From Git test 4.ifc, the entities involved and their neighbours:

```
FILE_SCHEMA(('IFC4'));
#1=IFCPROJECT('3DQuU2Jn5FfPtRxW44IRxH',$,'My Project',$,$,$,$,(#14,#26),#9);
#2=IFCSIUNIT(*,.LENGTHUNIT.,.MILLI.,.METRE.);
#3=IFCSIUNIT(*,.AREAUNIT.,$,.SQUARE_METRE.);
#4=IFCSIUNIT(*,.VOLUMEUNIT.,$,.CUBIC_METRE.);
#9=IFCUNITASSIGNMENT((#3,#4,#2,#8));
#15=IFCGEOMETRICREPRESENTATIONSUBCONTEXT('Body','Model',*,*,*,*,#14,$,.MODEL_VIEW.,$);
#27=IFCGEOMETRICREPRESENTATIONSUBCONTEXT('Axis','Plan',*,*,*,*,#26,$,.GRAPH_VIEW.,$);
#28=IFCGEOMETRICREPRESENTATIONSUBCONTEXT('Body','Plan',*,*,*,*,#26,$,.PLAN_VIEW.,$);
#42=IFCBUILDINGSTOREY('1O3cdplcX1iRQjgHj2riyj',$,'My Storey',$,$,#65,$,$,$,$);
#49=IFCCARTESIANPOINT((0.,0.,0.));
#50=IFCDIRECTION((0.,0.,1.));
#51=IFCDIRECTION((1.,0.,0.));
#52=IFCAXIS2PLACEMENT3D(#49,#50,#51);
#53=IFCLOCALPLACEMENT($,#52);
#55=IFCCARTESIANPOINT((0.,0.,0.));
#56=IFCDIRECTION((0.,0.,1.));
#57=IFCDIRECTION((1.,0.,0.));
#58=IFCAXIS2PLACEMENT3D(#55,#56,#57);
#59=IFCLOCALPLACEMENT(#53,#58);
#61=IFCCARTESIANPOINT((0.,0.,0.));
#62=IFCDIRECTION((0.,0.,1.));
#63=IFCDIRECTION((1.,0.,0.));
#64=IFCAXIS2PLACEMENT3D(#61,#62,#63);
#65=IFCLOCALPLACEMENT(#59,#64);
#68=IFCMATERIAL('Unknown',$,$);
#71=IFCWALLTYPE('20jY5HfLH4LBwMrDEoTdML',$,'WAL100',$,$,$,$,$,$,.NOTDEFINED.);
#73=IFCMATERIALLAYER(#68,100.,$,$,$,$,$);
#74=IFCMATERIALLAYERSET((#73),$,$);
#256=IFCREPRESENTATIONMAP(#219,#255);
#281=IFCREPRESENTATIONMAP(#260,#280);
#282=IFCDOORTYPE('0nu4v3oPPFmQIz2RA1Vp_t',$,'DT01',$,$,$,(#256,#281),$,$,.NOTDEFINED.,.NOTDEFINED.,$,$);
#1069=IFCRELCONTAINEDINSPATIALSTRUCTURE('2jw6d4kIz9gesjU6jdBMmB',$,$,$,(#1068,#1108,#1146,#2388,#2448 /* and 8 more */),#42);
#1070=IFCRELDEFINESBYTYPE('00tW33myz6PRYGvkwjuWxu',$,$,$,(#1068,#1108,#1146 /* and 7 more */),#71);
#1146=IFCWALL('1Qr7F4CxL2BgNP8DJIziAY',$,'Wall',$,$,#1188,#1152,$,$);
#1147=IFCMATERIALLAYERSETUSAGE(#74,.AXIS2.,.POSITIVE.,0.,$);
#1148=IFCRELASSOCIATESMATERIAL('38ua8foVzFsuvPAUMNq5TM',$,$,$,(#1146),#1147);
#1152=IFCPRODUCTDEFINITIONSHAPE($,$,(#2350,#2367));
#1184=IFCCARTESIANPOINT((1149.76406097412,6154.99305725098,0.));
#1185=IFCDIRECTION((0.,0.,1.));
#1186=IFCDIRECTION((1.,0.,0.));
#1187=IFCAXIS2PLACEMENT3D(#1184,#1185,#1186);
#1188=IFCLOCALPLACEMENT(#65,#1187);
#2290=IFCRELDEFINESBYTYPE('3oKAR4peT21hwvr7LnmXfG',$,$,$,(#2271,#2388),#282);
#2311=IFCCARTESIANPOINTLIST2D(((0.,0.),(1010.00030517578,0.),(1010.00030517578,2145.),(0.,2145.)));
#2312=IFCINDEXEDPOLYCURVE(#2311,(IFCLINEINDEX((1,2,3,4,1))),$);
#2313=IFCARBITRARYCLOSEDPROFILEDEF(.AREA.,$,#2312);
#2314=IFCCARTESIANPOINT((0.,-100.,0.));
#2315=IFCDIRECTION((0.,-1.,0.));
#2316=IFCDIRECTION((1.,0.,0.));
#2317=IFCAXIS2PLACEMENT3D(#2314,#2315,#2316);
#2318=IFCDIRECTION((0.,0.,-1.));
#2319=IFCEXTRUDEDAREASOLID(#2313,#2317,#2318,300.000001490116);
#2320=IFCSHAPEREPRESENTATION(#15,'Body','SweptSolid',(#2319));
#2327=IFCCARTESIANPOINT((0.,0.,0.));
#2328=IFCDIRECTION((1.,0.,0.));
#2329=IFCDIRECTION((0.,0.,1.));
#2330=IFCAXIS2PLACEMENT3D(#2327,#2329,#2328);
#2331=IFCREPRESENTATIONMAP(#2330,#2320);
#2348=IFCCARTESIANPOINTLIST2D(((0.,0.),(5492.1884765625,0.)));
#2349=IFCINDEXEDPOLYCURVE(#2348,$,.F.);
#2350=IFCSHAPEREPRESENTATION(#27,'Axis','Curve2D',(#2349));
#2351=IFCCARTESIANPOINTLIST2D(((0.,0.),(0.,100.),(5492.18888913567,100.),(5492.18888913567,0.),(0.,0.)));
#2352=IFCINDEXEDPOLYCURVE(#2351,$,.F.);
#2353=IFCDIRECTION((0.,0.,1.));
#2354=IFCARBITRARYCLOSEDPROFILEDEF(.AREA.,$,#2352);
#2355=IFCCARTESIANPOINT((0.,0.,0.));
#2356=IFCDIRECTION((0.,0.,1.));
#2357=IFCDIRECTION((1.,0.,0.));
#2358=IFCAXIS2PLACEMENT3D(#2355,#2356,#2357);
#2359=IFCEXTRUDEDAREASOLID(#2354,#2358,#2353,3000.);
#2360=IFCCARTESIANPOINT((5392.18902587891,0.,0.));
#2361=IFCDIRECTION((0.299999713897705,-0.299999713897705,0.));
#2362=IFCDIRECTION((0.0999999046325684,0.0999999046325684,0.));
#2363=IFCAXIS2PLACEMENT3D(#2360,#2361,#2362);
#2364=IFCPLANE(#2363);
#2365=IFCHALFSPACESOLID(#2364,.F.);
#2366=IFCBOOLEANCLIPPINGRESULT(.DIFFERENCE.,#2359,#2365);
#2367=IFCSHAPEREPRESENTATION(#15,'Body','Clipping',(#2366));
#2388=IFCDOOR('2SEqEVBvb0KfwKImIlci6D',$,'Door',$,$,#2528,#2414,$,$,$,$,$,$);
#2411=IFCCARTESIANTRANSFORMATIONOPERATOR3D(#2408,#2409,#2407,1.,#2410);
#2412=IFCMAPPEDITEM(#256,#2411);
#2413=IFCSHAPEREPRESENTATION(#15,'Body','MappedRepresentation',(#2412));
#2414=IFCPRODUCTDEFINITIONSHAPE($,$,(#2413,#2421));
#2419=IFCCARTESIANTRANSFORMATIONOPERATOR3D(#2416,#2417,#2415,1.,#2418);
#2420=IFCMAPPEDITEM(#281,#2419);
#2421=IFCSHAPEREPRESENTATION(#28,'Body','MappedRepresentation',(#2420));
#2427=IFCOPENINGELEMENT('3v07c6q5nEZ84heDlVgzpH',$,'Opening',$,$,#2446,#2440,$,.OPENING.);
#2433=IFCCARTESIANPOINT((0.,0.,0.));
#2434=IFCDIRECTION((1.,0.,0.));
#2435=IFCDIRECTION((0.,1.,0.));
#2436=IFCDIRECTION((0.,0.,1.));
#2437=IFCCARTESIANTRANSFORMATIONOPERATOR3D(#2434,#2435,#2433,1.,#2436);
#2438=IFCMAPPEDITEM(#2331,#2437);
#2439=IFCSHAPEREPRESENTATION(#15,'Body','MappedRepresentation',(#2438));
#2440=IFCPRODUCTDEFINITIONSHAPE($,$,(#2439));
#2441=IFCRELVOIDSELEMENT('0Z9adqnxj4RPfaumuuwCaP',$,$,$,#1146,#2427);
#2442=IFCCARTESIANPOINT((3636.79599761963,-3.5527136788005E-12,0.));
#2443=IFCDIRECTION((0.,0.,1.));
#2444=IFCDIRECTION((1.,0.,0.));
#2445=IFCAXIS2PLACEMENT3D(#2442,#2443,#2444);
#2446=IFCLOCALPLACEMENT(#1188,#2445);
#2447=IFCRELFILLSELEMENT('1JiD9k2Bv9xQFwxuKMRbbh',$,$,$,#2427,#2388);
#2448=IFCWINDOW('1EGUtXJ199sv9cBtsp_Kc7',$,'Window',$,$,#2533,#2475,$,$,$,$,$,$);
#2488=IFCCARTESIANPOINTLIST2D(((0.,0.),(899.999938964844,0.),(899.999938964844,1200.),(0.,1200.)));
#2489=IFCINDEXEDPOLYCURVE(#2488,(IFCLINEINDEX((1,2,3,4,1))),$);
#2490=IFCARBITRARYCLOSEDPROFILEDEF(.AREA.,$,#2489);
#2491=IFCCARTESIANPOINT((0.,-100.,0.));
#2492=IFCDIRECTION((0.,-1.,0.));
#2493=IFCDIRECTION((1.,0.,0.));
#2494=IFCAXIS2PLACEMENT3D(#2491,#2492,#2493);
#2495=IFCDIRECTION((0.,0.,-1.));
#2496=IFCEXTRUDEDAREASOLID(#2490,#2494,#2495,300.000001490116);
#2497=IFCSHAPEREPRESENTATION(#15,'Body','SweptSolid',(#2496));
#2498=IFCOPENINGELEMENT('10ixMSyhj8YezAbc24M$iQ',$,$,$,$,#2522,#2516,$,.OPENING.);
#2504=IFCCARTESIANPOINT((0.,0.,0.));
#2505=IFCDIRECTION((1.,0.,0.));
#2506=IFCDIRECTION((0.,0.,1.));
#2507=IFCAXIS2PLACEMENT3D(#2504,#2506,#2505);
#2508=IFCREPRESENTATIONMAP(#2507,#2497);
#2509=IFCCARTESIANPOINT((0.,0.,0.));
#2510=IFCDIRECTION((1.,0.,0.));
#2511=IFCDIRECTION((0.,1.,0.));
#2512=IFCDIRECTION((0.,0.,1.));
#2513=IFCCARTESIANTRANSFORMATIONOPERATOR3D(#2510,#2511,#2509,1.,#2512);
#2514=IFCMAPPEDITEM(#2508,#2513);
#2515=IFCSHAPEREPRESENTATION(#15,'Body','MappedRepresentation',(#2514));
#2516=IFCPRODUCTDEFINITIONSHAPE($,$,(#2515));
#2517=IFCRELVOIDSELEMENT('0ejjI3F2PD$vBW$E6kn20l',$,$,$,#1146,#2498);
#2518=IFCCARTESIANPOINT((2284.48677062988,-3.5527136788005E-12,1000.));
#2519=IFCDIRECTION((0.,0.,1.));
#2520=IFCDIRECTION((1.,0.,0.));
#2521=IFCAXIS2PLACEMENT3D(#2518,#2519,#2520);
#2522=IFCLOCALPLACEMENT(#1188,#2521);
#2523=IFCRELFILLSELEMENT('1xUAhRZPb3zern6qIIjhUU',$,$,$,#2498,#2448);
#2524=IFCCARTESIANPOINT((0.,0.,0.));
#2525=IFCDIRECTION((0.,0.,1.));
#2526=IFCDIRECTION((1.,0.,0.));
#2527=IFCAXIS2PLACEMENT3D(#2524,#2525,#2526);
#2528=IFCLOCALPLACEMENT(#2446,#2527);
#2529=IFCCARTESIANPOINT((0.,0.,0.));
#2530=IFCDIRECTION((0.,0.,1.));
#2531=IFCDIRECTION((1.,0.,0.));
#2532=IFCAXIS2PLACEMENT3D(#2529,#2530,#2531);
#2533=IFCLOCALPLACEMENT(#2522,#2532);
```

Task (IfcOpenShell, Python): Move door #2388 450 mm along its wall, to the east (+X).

```python
import ifcopenshell
import ifcopenshell.api.geometry
import ifcopenshell.util.placement

model = ifcopenshell.open("Git test 4.ifc")

door = model.by_guid("2SEqEVBvb0KfwKImIlci6D")
opening = door.FillsVoids[0].RelatingOpeningElement
wall = opening.VoidsElements[0].RelatingBuildingElement

wall_matrix = ifcopenshell.util.placement.get_local_placement(wall.ObjectPlacement)
shift = wall_matrix[:3, 0] * 450.0
before = ifcopenshell.util.placement.get_local_placement(door.ObjectPlacement)[:3, 3].copy()

# The door is placed relative to its opening, so it follows when the opening moves.
matrix = ifcopenshell.util.placement.get_local_placement(opening.ObjectPlacement)
matrix[:3, 3] += shift
ifcopenshell.api.geometry.edit_object_placement(
    model, product=opening, matrix=matrix, is_si=False, should_transform_children=True
)

after = ifcopenshell.util.placement.get_local_placement(door.ObjectPlacement)[:3, 3]
print("door moved by", (after - before).round(3) + 0.0)

model.write("Git test 4_rev.ifc")
```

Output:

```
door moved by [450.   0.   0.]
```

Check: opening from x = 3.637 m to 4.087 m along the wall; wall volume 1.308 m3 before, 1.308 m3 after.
